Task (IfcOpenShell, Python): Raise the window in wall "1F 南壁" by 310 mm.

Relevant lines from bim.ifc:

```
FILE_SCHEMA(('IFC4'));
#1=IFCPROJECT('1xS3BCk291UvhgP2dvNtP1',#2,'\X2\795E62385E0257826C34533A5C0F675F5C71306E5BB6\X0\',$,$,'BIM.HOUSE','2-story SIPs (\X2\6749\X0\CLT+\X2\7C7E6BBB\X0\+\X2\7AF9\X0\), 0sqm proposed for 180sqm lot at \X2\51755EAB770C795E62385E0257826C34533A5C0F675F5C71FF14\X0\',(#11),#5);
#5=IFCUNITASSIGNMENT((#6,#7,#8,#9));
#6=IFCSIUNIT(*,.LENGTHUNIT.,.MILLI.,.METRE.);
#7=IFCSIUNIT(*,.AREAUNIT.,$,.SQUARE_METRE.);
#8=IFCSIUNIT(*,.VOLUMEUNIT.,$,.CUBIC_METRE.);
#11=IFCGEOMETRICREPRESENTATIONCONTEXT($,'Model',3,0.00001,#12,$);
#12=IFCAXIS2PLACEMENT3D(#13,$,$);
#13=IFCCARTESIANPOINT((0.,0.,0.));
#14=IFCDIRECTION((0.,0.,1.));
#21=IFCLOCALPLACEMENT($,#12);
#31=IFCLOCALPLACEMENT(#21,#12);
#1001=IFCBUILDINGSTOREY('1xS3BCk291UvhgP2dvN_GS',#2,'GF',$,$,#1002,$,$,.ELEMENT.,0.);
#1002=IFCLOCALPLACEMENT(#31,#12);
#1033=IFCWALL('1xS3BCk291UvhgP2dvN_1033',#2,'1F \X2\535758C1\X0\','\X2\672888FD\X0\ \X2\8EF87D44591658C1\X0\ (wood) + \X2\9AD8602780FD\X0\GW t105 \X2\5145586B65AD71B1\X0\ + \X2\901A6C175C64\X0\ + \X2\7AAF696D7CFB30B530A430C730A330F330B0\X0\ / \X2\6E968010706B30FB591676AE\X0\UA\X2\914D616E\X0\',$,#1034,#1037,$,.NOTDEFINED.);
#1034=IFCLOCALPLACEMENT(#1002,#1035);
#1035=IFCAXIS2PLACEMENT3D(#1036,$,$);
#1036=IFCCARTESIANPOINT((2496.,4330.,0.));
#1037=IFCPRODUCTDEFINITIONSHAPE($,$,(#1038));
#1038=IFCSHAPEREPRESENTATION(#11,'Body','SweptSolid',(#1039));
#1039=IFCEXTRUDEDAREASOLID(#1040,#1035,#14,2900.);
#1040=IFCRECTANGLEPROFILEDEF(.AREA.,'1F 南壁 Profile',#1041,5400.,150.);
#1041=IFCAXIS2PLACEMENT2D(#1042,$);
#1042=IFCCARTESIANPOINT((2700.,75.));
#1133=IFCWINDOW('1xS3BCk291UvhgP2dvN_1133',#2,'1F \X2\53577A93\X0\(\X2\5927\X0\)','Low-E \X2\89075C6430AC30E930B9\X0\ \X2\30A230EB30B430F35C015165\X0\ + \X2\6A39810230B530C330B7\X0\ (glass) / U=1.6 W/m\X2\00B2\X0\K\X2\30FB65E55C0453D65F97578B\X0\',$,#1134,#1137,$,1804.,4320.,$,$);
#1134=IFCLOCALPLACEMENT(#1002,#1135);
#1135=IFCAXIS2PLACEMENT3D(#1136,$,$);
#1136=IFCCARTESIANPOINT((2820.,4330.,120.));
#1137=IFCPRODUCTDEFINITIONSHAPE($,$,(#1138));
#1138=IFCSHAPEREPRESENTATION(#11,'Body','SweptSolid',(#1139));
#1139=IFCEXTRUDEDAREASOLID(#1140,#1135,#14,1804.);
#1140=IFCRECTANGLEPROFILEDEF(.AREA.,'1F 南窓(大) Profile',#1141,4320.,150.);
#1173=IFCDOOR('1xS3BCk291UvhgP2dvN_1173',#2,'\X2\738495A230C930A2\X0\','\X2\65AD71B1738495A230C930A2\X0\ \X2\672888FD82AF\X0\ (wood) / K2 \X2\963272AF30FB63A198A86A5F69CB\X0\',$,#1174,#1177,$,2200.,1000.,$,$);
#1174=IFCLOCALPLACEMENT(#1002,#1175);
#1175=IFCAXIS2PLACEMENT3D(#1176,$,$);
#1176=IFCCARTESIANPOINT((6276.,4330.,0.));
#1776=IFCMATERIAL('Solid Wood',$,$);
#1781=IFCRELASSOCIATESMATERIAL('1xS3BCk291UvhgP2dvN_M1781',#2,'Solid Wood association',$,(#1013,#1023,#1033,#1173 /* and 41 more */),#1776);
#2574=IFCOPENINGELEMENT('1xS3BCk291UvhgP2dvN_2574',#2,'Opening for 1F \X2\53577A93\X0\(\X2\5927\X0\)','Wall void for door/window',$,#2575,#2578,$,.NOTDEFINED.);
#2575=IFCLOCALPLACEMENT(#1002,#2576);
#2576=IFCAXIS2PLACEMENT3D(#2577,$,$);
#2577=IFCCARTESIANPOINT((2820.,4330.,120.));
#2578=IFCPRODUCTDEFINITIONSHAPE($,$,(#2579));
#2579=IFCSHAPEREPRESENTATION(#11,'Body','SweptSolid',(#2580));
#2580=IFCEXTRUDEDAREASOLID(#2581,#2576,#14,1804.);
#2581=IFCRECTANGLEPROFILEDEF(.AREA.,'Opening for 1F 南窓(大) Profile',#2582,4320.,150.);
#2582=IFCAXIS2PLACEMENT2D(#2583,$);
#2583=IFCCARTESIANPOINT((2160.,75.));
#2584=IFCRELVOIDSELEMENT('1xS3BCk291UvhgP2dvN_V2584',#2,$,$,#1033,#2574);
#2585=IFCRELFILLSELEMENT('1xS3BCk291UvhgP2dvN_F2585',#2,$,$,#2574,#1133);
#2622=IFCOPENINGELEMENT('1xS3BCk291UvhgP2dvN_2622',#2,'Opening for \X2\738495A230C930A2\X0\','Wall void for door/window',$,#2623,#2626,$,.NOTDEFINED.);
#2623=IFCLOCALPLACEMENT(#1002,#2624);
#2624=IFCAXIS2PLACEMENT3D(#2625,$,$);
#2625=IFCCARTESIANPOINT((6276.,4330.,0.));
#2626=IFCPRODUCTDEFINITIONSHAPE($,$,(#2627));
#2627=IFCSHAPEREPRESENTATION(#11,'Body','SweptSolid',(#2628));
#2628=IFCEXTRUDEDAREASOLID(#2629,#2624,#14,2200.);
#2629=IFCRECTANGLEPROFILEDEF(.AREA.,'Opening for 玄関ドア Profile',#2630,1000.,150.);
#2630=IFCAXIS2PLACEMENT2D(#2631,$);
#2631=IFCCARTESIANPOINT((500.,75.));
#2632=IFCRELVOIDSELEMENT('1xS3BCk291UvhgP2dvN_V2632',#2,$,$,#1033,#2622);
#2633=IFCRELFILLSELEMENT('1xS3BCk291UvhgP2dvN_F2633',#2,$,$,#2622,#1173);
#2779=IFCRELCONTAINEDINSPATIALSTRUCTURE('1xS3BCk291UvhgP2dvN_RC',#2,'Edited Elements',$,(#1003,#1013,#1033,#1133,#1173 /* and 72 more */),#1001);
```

```python
import numpy as np
import ifcopenshell
import ifcopenshell.api.geometry
import ifcopenshell.util.placement
import ifcopenshell.util.unit

model = ifcopenshell.open("bim.ifc")
unit_scale = ifcopenshell.util.unit.calculate_unit_scale(model)

window = model.by_guid("1xS3BCk291UvhgP2dvN_1133")
opening = window.FillsVoids[0].RelatingOpeningElement
dz = 310.0

shift = np.array([0.0, 0.0, dz])
# The window is not placed relative to its opening, so move both.
for product in (opening, window):
    matrix = ifcopenshell.util.placement.get_local_placement(product.ObjectPlacement)
    matrix[:3, 3] += shift
    ifcopenshell.api.geometry.edit_object_placement(model, product=product, matrix=matrix, is_si=False)

print(f"moved by {dz * unit_scale:+.3f} m")

model.write("bim_edited.ifc")
```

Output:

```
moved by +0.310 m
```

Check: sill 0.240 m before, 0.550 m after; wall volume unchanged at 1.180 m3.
